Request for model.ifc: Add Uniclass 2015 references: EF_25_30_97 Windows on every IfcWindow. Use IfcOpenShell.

First a look at what the model holds.

```python
import ifcopenshell

model = ifcopenshell.open("model.ifc")
print(model.schema)
print("classifications:", [c.Name for c in model.by_type("IfcClassification")])
for ifc_class in ("IfcDoor", "IfcRoof", "IfcStair", "IfcWall", "IfcWindow"):
    print(ifc_class, len(model.by_type(ifc_class)))
```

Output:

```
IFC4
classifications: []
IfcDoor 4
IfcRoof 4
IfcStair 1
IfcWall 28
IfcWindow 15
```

```python
import ifcopenshell
import ifcopenshell.api.classification

model = ifcopenshell.open("model.ifc")

system = ifcopenshell.api.classification.add_classification(model, classification="Uniclass 2015")

codes = {
    "IfcWindow": ("EF_25_30_97", "Windows"),
}
for ifc_class, (code, name) in codes.items():
    products = model.by_type(ifc_class)
    ifcopenshell.api.classification.add_reference(
        model, products=products, classification=system, identification=code, name=name
    )
    print(code, len(products))

model.write("model-out.ifc")
```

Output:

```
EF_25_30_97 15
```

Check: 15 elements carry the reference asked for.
